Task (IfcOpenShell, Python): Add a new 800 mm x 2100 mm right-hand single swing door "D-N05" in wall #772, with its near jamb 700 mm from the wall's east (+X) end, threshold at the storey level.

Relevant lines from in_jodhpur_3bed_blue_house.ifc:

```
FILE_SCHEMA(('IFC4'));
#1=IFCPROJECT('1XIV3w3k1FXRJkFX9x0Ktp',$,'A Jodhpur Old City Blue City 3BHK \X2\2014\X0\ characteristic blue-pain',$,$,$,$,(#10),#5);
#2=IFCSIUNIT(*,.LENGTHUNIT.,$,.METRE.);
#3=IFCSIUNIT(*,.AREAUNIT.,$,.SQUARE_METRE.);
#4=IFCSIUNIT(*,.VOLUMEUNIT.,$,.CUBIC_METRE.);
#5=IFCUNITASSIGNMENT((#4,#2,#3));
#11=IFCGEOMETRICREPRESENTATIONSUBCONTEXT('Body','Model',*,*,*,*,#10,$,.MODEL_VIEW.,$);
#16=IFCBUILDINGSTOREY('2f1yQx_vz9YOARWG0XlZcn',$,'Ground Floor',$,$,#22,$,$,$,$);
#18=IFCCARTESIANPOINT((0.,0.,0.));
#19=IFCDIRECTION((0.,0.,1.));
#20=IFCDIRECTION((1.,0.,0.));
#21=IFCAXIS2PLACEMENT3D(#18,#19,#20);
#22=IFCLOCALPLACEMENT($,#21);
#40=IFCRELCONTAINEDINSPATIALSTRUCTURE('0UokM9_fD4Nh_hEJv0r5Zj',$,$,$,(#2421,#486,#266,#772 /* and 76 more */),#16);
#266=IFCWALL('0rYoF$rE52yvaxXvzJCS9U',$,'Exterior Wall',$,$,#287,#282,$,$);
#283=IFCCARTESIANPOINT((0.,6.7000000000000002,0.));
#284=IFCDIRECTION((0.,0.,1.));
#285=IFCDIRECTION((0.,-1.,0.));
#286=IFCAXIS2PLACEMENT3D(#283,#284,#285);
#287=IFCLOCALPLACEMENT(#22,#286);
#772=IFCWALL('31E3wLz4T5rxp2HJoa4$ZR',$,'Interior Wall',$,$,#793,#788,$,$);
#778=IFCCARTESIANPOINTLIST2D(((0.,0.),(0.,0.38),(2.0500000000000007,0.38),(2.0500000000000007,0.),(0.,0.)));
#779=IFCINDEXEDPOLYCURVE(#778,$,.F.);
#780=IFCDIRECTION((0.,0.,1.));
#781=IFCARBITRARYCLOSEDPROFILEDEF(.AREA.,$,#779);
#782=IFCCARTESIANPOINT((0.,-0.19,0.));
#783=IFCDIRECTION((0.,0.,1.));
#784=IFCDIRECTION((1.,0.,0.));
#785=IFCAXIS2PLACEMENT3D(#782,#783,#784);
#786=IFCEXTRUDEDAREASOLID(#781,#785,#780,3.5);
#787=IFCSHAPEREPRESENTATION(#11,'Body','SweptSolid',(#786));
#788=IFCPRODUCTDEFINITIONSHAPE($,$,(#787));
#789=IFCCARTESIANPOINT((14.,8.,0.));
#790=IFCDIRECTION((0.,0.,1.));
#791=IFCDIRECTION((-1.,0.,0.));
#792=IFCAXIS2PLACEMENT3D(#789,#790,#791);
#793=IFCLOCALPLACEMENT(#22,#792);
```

```python
import numpy as np
import ifcopenshell
import ifcopenshell.api.feature
import ifcopenshell.api.geometry
import ifcopenshell.api.root
import ifcopenshell.api.spatial
import ifcopenshell.geom
import ifcopenshell.util.element
import ifcopenshell.util.placement
import ifcopenshell.util.representation
import ifcopenshell.util.shape
import ifcopenshell.util.unit

model = ifcopenshell.open("in_jodhpur_3bed_blue_house.ifc")
unit_scale = ifcopenshell.util.unit.calculate_unit_scale(model)
settings = ifcopenshell.geom.settings()


def volume(element):
    """Net volume in cubic metres, openings subtracted."""
    shape = ifcopenshell.geom.create_shape(settings, element)
    return ifcopenshell.util.shape.get_volume(shape.geometry)


wall = model.by_guid("31E3wLz4T5rxp2HJoa4$ZR")
storey = ifcopenshell.util.element.get_container(wall, ifc_class="IfcBuildingStorey")
context = ifcopenshell.util.representation.get_context(model, "Model", "Body", "MODEL_VIEW")
before = volume(wall)

width, height, from_end, sill = 0.8, 2.1, 0.7, 0.0  # metres

# The wall runs along its own X axis, and the end named is its -X end.
wall_shape = ifcopenshell.geom.create_shape(settings, wall)
x, y, z = ifcopenshell.util.shape.get_vertices(wall_shape.geometry).T
start = x.min() + from_end
face, thickness = float(y.min()), float(y.max() - y.min())
wall_matrix = ifcopenshell.util.placement.get_local_placement(wall.ObjectPlacement)
level = ifcopenshell.util.placement.get_local_placement(storey.ObjectPlacement)[2, 3]


def in_wall(x, y):
    """Placement at x, y metres in the wall's axes, at sill height."""
    matrix = wall_matrix.copy()
    matrix[:, 3] = wall_matrix @ np.array([x / unit_scale, y / unit_scale, 0.0, 1.0])
    matrix[2, 3] = level + sill / unit_scale
    return matrix


# Opening: a box that overshoots both wall faces by 50 mm.
opening = ifcopenshell.api.root.create_entity(model, ifc_class="IfcOpeningElement", predefined_type="OPENING")
box = ifcopenshell.api.geometry.add_wall_representation(
    model, context=context, length=width, height=height, thickness=thickness + 0.1
)
ifcopenshell.api.geometry.assign_representation(model, product=opening, representation=box)
ifcopenshell.api.geometry.edit_object_placement(model, product=opening, matrix=in_wall(start, face - 0.05), is_si=False)
ifcopenshell.api.feature.add_feature(model, feature=opening, element=wall)

door = ifcopenshell.api.root.create_entity(model, ifc_class="IfcDoor", name="D-N05", predefined_type="DOOR")
door.OverallWidth, door.OverallHeight = width / unit_scale, height / unit_scale
door.OperationType = "SINGLE_SWING_RIGHT"
body = ifcopenshell.api.geometry.add_door_representation(
    model,
    context=context,
    overall_width=door.OverallWidth,
    overall_height=door.OverallHeight,
    operation_type="SINGLE_SWING_RIGHT",
    lining_properties={"LiningDepth": thickness / unit_scale, "ThresholdDepth": thickness / unit_scale},
)
ifcopenshell.api.geometry.assign_representation(model, product=door, representation=body)
ifcopenshell.api.spatial.assign_container(model, products=[door], relating_structure=storey)
ifcopenshell.api.feature.add_filling(model, opening=opening, element=door)

# The lining spans the wall, so the door starts at the wall face.
ifcopenshell.api.geometry.edit_object_placement(model, product=door, matrix=in_wall(start, face), is_si=False)

after = volume(wall)

print(f"wall volume {before:.3f} -> {after:.3f} m3")

model.write("in_jodhpur_3bed_blue_house_updated.ifc")
```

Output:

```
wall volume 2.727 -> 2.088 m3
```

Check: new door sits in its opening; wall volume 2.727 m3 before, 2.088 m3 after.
